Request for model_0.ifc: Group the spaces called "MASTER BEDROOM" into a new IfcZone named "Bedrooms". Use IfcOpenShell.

First a look at what the model holds.

```python
import ifcopenshell

model = ifcopenshell.open("model_0.ifc")
print(model.schema)
seen = {}
for space in model.by_type("IfcSpace"):
    seen[space.LongName] = seen.get(space.LongName, 0) + 1
for name, count in sorted(seen.items(), key=str):
    print(count, "x", name)
print("zones:", [z.Name for z in model.by_type("IfcZone")][:20])
```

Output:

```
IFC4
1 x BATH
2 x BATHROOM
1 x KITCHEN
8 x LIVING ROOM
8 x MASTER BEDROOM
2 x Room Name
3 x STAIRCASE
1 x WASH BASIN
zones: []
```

```python
import ifcopenshell
import ifcopenshell.api.group
import ifcopenshell.api.root

model = ifcopenshell.open("model_0.ifc")

names = {"MASTER BEDROOM"}
spaces = [s for s in model.by_type("IfcSpace") if s.LongName in names]

zone = ifcopenshell.api.root.create_entity(model, ifc_class="IfcZone", name="Bedrooms")
ifcopenshell.api.group.assign_group(model, products=spaces, group=zone)
print(len(spaces), "spaces in", zone.Name)

model.write("model_0_rev.ifc")
```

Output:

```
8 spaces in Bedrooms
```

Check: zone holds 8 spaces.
